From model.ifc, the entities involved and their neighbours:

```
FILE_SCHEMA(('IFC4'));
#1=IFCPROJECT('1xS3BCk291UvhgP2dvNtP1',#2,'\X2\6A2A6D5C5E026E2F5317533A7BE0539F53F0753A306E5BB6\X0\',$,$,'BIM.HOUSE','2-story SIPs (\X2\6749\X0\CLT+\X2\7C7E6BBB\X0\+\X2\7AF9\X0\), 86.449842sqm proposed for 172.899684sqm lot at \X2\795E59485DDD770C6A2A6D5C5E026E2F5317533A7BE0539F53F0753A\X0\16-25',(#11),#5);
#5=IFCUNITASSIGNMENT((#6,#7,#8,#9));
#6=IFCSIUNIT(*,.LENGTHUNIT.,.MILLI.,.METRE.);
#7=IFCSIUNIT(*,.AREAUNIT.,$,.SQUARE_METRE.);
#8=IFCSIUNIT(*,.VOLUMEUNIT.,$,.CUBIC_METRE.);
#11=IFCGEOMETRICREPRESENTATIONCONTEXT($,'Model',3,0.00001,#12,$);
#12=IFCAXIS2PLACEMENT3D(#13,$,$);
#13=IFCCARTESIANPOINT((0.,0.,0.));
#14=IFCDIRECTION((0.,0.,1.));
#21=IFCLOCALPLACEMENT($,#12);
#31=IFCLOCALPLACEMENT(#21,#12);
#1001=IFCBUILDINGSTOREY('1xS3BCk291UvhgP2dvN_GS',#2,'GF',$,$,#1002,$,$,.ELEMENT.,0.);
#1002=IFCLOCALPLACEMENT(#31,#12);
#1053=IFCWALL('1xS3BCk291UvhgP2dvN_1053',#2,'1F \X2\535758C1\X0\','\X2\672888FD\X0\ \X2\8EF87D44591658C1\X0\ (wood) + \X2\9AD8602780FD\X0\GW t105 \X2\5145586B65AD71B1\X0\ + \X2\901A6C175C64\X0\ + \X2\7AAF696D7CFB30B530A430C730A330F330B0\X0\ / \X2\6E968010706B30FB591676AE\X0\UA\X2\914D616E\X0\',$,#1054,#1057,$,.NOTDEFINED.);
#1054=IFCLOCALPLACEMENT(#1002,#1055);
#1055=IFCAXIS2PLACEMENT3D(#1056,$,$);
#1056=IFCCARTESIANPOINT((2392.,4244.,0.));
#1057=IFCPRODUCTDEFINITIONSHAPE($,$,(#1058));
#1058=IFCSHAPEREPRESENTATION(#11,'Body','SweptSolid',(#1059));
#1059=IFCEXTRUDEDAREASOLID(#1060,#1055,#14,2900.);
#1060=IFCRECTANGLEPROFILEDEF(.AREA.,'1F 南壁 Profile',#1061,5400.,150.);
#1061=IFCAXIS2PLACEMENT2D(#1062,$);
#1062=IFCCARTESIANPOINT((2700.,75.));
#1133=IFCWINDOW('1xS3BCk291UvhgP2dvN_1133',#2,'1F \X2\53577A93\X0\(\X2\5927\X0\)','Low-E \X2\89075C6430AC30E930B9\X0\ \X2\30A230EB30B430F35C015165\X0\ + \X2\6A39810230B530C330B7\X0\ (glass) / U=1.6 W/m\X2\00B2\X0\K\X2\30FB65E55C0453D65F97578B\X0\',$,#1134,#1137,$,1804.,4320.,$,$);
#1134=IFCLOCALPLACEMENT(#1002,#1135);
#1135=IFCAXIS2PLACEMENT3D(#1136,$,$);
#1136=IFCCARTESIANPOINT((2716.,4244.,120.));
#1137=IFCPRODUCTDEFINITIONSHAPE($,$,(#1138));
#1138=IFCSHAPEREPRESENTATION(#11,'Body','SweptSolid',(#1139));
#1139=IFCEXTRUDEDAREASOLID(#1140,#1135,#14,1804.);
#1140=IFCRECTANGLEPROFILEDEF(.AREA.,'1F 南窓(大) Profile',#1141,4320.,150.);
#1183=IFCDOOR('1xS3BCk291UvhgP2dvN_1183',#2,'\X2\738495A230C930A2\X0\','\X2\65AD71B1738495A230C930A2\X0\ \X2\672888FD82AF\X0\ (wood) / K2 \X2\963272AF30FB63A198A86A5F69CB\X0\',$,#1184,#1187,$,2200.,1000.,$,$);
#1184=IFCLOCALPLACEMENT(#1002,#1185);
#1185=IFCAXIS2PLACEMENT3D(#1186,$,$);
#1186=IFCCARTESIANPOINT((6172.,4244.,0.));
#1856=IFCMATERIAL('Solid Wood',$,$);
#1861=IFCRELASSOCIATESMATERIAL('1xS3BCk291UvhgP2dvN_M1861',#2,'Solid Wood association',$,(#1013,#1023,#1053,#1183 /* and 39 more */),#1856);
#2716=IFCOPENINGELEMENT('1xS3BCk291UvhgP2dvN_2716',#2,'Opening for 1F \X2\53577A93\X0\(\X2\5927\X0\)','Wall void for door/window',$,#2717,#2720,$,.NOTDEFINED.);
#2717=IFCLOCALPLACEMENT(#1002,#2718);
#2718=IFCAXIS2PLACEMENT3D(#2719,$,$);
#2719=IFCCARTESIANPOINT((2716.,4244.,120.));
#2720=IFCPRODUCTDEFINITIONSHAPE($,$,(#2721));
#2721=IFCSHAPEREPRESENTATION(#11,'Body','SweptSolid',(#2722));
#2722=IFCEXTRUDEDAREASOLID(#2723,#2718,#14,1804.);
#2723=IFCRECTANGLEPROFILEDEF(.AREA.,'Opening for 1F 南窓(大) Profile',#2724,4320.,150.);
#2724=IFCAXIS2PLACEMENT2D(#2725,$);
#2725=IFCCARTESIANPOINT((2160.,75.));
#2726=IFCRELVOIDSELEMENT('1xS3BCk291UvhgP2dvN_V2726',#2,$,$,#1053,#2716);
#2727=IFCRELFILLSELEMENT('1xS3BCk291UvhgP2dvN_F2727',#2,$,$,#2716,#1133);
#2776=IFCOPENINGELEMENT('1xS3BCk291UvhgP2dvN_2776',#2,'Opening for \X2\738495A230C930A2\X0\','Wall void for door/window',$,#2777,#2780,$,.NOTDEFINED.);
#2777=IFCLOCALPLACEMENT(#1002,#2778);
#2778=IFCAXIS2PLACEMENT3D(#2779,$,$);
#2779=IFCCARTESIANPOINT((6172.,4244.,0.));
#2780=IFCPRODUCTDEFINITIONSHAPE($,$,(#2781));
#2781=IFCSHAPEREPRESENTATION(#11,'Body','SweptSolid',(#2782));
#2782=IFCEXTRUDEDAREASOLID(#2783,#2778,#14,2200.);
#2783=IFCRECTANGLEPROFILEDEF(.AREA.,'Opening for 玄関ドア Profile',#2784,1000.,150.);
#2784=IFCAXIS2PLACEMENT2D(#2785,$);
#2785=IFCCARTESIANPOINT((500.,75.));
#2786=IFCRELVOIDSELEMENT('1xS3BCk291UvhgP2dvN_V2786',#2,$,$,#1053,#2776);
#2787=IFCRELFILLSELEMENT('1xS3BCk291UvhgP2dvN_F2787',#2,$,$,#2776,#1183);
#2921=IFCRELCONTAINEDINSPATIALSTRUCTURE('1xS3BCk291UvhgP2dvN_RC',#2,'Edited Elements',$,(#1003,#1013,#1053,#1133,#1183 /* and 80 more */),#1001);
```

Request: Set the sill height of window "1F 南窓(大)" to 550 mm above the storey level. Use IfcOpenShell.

```python
import numpy as np
import ifcopenshell
import ifcopenshell.api.geometry
import ifcopenshell.geom
import ifcopenshell.util.element
import ifcopenshell.util.placement
import ifcopenshell.util.shape
import ifcopenshell.util.unit

model = ifcopenshell.open("model.ifc")
unit_scale = ifcopenshell.util.unit.calculate_unit_scale(model)

window = model.by_guid("1xS3BCk291UvhgP2dvN_1133")
opening = window.FillsVoids[0].RelatingOpeningElement
storey = ifcopenshell.util.element.get_container(window, ifc_class="IfcBuildingStorey")
level = ifcopenshell.util.placement.get_local_placement(storey.ObjectPlacement)[2, 3]

# The opening's origin need not be at the sill, so measure its lowest point.
shape = ifcopenshell.geom.create_shape(ifcopenshell.geom.settings(), opening)
bottom = ifcopenshell.util.shape.get_shape_bottom_elevation(shape, shape.geometry) / unit_scale
dz = level + 0.55 / unit_scale - bottom

shift = np.array([0.0, 0.0, dz])
# The window is not placed relative to its opening, so move both.
for product in (opening, window):
    matrix = ifcopenshell.util.placement.get_local_placement(product.ObjectPlacement)
    matrix[:3, 3] += shift
    ifcopenshell.api.geometry.edit_object_placement(model, product=product, matrix=matrix, is_si=False)

print(f"moved by {dz * unit_scale:+.3f} m")

model.write("model_rev.ifc")
```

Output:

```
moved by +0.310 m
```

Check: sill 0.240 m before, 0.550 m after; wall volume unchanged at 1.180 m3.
